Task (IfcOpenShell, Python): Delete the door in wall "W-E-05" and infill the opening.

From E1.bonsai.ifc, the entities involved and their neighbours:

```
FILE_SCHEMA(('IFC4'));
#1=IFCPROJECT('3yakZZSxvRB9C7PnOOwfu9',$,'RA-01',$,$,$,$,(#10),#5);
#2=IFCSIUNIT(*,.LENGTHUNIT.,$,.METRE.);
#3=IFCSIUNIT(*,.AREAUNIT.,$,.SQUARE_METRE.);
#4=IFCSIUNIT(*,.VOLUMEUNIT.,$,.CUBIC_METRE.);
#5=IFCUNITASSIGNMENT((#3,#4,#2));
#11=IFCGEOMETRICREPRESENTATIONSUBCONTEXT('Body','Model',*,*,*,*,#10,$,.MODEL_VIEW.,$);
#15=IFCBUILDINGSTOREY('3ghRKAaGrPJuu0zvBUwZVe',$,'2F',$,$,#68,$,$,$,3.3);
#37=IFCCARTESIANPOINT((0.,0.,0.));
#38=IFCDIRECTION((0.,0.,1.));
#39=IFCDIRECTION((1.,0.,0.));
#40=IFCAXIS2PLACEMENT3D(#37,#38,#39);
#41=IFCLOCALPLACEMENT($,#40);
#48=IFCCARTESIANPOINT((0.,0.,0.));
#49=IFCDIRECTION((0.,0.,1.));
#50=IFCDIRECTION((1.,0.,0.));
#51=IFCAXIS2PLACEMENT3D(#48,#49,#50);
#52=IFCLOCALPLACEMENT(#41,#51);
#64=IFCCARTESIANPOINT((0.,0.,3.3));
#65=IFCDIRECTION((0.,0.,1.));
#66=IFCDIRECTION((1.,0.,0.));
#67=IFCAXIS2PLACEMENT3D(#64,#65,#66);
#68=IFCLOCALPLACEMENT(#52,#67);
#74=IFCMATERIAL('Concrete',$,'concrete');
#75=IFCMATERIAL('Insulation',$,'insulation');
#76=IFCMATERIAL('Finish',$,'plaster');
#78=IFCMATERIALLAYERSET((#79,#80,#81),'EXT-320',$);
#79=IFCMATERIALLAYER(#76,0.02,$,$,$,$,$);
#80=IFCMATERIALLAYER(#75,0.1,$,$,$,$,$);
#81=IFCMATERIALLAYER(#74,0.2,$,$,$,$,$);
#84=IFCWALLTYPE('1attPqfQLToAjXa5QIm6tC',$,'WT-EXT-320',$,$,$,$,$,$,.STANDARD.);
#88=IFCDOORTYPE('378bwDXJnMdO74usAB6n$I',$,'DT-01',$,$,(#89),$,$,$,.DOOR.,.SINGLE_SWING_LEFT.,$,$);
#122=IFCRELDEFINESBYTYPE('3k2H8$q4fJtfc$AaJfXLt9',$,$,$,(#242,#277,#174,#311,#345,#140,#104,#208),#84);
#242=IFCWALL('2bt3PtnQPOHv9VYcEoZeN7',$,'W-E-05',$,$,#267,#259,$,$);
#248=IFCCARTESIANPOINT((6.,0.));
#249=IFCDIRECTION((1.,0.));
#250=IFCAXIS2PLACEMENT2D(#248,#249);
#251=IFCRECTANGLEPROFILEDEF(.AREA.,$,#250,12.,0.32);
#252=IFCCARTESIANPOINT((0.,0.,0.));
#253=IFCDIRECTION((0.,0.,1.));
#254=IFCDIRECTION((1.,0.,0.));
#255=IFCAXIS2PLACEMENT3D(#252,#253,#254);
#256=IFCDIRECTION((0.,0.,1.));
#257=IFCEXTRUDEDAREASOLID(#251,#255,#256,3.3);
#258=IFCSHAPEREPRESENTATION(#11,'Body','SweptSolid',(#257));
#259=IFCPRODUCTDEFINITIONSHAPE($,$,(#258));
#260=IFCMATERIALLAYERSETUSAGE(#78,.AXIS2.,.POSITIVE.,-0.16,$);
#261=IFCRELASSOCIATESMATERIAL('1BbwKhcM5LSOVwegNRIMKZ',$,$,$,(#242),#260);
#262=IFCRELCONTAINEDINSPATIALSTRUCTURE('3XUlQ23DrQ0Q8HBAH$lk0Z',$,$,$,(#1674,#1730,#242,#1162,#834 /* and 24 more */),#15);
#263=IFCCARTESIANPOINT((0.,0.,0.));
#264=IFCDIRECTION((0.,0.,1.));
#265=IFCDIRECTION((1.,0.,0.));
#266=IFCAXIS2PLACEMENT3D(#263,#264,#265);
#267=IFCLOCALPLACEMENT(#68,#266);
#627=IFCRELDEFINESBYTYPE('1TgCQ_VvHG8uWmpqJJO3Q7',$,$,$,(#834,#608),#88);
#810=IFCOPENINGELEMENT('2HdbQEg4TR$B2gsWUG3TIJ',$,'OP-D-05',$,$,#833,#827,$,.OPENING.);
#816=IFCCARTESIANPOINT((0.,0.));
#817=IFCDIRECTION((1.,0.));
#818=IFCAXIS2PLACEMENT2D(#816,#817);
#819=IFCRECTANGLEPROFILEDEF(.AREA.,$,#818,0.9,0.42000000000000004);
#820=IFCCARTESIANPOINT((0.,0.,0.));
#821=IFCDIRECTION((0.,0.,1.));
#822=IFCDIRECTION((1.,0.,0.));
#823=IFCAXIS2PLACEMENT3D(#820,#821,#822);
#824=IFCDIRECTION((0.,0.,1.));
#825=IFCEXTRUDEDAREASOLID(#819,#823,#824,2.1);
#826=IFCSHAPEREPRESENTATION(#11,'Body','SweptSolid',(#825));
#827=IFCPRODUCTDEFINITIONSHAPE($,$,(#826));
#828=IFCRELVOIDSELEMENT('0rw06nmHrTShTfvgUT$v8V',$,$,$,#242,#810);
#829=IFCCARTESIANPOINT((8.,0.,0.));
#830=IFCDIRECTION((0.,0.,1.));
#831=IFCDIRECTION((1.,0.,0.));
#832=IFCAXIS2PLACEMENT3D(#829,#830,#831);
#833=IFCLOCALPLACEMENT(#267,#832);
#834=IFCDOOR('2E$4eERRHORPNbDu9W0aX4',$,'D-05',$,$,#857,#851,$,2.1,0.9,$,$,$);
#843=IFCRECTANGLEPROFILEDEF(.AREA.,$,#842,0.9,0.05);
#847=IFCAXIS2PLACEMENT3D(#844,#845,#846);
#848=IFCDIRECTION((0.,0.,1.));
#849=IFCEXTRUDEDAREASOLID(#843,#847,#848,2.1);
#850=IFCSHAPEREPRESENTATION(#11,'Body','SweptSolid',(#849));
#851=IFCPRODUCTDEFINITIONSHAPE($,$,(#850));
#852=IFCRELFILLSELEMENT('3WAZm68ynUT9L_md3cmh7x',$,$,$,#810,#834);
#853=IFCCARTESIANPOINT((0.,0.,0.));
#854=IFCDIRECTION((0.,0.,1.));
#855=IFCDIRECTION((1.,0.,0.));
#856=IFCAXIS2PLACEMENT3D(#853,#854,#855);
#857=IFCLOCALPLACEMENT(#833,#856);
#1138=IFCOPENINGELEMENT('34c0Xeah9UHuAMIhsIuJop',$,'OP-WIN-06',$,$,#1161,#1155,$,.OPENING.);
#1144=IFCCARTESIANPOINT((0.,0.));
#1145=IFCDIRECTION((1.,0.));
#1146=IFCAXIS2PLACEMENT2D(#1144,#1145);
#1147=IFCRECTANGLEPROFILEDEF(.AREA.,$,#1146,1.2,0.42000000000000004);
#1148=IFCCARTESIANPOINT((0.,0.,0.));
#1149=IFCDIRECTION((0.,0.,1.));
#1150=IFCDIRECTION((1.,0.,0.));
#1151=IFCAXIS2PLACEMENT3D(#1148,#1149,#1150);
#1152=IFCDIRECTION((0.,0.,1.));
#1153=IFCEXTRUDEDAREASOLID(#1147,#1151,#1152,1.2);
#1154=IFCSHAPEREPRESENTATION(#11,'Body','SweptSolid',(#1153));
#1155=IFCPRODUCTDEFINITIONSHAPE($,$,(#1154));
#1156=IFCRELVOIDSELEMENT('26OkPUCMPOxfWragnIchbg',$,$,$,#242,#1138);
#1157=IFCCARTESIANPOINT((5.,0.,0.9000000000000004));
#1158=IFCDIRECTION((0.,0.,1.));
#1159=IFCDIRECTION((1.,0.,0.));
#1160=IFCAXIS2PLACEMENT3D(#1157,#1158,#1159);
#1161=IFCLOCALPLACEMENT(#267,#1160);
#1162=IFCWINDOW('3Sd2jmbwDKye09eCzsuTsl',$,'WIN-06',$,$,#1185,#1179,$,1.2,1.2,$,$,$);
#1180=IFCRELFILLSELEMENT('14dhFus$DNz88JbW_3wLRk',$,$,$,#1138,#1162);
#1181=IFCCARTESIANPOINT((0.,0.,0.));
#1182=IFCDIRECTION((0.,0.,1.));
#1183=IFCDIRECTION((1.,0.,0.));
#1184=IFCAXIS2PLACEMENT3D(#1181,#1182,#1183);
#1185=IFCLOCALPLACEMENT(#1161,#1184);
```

```python
import ifcopenshell
import ifcopenshell.api.feature
import ifcopenshell.api.root
import ifcopenshell.geom
import ifcopenshell.util.shape

model = ifcopenshell.open("E1.bonsai.ifc")
settings = ifcopenshell.geom.settings()


def volume(element):
    """Net volume in cubic metres, openings subtracted."""
    shape = ifcopenshell.geom.create_shape(settings, element)
    return ifcopenshell.util.shape.get_volume(shape.geometry)


door = model.by_id(834)
opening = door.FillsVoids[0].RelatingOpeningElement
wall = opening.VoidsElements[0].RelatingBuildingElement
before = volume(wall)

ifcopenshell.api.root.remove_product(model, product=door)
ifcopenshell.api.feature.remove_feature(model, feature=opening)

after = volume(wall)

print(f"wall volume {before:.3f} -> {after:.3f} m3")

model.write("E1.bonsai_rev.ifc")
```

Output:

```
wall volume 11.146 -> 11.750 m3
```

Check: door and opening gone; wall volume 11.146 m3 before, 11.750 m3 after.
